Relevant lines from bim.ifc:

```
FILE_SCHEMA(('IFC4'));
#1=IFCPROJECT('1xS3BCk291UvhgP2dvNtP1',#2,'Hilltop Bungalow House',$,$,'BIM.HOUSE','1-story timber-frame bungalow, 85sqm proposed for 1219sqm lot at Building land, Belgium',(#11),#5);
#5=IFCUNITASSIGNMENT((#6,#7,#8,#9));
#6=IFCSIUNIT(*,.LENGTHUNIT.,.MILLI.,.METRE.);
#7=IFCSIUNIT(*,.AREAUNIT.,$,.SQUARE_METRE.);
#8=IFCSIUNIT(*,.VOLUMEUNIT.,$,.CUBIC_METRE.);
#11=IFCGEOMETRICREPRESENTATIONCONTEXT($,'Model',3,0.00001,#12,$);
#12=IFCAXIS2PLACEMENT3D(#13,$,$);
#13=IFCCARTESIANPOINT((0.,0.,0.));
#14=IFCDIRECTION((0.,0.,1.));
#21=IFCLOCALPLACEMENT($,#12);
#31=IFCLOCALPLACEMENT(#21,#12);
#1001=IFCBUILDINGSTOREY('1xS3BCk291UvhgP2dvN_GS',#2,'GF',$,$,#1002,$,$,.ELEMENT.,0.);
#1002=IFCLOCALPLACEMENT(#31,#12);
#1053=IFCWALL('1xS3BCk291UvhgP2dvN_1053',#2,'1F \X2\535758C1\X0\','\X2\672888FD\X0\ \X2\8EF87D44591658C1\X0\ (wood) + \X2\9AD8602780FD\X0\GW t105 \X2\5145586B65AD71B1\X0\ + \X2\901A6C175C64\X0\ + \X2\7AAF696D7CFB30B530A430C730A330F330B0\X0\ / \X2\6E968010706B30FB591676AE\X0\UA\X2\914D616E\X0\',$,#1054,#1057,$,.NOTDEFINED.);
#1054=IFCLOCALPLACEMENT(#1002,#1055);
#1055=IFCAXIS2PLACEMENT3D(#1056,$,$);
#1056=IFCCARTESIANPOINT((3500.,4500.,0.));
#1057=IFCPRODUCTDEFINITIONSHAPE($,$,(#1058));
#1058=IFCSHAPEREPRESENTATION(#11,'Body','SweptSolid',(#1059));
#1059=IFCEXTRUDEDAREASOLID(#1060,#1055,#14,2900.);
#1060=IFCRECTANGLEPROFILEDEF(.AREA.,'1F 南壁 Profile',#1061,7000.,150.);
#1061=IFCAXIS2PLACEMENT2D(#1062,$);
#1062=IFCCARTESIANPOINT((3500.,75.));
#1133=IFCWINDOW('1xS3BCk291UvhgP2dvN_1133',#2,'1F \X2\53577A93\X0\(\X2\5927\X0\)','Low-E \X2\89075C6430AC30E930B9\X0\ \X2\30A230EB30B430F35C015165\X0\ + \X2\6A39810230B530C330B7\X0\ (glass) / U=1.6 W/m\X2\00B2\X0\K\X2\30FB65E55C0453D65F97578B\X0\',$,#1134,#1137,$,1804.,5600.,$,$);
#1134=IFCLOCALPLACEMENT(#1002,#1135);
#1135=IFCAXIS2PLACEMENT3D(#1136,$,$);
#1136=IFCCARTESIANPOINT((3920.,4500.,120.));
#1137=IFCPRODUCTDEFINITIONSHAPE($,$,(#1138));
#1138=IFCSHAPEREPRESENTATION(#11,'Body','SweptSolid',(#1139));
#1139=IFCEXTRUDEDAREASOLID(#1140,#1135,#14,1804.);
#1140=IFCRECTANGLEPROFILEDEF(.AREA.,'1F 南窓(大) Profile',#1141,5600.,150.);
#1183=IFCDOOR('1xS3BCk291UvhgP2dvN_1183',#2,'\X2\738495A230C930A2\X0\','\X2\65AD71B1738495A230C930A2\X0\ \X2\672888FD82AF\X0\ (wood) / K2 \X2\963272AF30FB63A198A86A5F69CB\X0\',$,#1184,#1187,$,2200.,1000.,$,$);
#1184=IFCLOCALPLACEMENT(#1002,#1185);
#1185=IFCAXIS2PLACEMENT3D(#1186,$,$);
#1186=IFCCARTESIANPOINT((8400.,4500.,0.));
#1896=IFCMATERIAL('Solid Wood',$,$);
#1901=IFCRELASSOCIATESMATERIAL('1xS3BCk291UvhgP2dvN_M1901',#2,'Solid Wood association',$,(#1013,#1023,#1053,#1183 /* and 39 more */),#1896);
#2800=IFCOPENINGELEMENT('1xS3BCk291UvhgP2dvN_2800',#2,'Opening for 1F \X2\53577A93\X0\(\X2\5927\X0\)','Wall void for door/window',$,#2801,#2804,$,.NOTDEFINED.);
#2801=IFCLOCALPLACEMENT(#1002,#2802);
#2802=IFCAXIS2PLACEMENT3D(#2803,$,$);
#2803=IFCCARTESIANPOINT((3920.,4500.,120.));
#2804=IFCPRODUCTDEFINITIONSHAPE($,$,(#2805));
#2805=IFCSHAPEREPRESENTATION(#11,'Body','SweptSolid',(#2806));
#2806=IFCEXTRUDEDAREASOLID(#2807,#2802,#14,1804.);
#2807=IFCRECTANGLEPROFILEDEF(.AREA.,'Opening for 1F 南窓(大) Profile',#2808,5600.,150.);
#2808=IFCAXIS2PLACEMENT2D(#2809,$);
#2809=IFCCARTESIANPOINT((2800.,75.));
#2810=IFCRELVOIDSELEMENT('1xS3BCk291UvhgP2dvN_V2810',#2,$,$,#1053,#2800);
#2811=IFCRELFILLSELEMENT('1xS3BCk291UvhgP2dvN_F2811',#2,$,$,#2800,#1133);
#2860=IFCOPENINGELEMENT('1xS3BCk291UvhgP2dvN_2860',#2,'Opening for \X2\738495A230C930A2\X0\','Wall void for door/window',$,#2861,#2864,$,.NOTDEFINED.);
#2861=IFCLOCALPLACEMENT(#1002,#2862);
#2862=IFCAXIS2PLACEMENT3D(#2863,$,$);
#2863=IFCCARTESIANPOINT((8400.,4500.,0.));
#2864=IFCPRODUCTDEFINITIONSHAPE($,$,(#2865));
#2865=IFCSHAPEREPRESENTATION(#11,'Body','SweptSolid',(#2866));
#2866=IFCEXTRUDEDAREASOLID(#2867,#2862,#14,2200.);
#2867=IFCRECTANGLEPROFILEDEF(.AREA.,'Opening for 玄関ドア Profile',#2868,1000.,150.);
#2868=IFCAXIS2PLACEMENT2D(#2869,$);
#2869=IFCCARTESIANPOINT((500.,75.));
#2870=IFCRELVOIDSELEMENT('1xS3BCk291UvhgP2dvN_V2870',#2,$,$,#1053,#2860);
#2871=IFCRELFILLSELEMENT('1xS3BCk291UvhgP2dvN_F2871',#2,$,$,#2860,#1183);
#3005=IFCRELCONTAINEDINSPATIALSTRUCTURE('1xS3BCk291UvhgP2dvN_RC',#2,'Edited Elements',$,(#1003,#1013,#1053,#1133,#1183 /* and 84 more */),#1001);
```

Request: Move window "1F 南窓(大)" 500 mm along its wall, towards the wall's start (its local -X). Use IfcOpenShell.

```python
import ifcopenshell
import ifcopenshell.api.geometry
import ifcopenshell.util.placement

model = ifcopenshell.open("bim.ifc")

window = model.by_guid("1xS3BCk291UvhgP2dvN_1133")
opening = window.FillsVoids[0].RelatingOpeningElement
wall = opening.VoidsElements[0].RelatingBuildingElement

wall_matrix = ifcopenshell.util.placement.get_local_placement(wall.ObjectPlacement)
shift = wall_matrix[:3, 0] * -500.0
before = ifcopenshell.util.placement.get_local_placement(window.ObjectPlacement)[:3, 3].copy()

# The window is not placed relative to its opening, so move both.
for product in (opening, window):
    matrix = ifcopenshell.util.placement.get_local_placement(product.ObjectPlacement)
    matrix[:3, 3] += shift
    ifcopenshell.api.geometry.edit_object_placement(model, product=product, matrix=matrix, is_si=False)

after = ifcopenshell.util.placement.get_local_placement(window.ObjectPlacement)[:3, 3]
print("window moved by", (after - before).round(3) + 0.0)

model.write("bim_rev.ifc")
```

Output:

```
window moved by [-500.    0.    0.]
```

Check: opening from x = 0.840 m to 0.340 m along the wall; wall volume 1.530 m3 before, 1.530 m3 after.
